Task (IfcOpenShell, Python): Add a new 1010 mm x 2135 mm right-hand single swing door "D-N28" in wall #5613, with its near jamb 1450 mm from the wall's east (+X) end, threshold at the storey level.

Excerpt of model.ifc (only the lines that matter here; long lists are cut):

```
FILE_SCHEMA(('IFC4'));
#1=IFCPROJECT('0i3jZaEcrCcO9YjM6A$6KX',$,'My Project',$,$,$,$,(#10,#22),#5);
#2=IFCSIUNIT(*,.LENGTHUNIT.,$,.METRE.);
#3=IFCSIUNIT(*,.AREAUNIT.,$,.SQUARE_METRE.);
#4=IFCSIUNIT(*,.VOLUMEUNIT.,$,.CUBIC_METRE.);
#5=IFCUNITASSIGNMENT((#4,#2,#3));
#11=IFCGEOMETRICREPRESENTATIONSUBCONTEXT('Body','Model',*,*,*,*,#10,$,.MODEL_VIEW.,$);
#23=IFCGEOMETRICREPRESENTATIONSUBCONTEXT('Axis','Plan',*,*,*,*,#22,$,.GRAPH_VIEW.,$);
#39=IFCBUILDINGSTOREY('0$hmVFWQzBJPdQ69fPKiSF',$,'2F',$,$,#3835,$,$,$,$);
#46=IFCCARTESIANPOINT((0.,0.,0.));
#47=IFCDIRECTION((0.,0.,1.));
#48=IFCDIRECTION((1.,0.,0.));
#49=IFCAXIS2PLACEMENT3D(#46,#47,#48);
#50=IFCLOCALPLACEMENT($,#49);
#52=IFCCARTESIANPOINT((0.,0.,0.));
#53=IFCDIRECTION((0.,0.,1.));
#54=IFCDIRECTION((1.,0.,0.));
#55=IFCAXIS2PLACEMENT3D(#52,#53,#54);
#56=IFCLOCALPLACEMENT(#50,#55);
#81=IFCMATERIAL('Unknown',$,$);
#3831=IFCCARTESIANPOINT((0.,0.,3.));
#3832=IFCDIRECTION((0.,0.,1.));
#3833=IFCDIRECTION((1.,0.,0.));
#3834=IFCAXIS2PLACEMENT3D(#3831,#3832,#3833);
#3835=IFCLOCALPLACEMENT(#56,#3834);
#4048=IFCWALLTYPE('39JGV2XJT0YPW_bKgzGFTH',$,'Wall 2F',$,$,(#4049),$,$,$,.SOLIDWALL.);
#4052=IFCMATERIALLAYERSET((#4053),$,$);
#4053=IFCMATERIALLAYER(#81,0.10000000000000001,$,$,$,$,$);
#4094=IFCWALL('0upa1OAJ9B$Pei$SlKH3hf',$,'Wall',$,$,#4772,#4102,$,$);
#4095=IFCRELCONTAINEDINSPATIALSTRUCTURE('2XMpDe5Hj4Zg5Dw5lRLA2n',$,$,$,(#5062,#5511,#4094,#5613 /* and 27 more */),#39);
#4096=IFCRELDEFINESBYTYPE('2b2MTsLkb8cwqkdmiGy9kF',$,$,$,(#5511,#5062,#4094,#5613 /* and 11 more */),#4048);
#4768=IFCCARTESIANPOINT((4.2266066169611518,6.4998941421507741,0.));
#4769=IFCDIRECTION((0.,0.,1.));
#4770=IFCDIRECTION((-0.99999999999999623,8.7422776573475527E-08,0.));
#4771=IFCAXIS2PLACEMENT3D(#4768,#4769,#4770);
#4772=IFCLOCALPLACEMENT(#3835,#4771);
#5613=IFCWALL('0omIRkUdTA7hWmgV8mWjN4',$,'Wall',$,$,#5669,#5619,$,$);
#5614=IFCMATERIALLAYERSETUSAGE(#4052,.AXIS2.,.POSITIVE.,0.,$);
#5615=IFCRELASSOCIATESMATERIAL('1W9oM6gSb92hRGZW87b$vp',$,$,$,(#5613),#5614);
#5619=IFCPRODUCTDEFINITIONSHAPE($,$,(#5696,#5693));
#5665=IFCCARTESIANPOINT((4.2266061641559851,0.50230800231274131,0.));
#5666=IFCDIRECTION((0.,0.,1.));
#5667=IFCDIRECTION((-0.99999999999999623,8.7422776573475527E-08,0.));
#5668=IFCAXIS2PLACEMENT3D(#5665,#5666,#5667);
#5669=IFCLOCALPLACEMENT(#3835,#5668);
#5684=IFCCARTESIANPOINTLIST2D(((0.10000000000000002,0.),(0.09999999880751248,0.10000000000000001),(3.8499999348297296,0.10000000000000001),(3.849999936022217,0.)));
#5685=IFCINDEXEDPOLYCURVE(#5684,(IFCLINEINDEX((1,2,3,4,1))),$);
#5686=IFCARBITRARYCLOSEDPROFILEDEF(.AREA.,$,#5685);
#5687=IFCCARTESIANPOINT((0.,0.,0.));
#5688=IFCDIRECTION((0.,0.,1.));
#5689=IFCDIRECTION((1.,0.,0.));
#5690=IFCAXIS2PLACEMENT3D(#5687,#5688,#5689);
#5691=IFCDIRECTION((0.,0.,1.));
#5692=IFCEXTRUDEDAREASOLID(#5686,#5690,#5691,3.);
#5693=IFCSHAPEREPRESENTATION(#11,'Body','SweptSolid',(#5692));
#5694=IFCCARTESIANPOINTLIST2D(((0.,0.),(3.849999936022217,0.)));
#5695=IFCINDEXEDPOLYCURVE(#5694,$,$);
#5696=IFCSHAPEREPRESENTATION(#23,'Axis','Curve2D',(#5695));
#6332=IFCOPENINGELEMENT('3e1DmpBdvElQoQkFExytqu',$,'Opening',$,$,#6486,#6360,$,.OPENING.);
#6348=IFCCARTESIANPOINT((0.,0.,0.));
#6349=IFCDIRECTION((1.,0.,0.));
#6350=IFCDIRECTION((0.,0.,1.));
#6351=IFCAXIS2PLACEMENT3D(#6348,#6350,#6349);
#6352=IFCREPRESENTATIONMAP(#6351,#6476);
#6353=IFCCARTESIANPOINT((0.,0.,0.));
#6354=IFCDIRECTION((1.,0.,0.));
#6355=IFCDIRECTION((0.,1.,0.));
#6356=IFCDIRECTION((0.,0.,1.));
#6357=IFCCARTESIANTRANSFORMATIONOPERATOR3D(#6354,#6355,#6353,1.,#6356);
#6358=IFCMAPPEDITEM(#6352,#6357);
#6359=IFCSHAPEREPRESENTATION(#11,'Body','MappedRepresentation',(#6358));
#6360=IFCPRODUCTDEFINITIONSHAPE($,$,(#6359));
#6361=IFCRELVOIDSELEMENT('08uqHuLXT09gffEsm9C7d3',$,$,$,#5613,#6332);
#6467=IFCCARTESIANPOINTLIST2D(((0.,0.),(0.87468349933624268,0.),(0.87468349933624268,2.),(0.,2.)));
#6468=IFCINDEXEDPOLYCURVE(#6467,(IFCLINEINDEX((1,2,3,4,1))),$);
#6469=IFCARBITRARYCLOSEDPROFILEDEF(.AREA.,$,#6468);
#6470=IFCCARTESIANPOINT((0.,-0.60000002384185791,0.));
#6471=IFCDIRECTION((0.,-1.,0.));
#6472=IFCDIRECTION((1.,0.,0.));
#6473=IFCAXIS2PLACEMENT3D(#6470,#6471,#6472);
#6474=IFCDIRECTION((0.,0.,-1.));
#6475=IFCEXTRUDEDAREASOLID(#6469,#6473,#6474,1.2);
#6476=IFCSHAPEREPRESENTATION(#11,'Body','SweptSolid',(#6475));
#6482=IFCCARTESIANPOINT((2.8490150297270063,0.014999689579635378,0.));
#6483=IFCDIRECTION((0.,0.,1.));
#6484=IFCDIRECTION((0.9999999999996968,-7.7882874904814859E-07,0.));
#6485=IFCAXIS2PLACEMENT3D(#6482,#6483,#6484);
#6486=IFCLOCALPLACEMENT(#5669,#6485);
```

```python
import numpy as np
import ifcopenshell
import ifcopenshell.api.feature
import ifcopenshell.api.geometry
import ifcopenshell.api.root
import ifcopenshell.api.spatial
import ifcopenshell.geom
import ifcopenshell.util.element
import ifcopenshell.util.placement
import ifcopenshell.util.representation
import ifcopenshell.util.shape
import ifcopenshell.util.unit

model = ifcopenshell.open("model.ifc")
unit_scale = ifcopenshell.util.unit.calculate_unit_scale(model)
settings = ifcopenshell.geom.settings()


def volume(element):
    """Net volume in cubic metres, openings subtracted."""
    shape = ifcopenshell.geom.create_shape(settings, element)
    return ifcopenshell.util.shape.get_volume(shape.geometry)


wall = model.by_guid("0omIRkUdTA7hWmgV8mWjN4")
storey = ifcopenshell.util.element.get_container(wall, ifc_class="IfcBuildingStorey")
context = ifcopenshell.util.representation.get_context(model, "Model", "Body", "MODEL_VIEW")
before = volume(wall)

width, height, from_end, sill = 1.01, 2.135, 1.45, 0.0  # metres

# The wall runs along its own X axis, and the end named is its -X end.
wall_shape = ifcopenshell.geom.create_shape(settings, wall)
x, y, z = ifcopenshell.util.shape.get_vertices(wall_shape.geometry).T
start = x.min() + from_end
face, thickness = float(y.min()), float(y.max() - y.min())
wall_matrix = ifcopenshell.util.placement.get_local_placement(wall.ObjectPlacement)
level = ifcopenshell.util.placement.get_local_placement(storey.ObjectPlacement)[2, 3]


def in_wall(x, y):
    """Placement at x, y metres in the wall's axes, at sill height."""
    matrix = wall_matrix.copy()
    matrix[:, 3] = wall_matrix @ np.array([x / unit_scale, y / unit_scale, 0.0, 1.0])
    matrix[2, 3] = level + sill / unit_scale
    return matrix


# Opening: a box that overshoots both wall faces by 50 mm.
opening = ifcopenshell.api.root.create_entity(model, ifc_class="IfcOpeningElement", predefined_type="OPENING")
box = ifcopenshell.api.geometry.add_wall_representation(
    model, context=context, length=width, height=height, thickness=thickness + 0.1
)
ifcopenshell.api.geometry.assign_representation(model, product=opening, representation=box)
ifcopenshell.api.geometry.edit_object_placement(model, product=opening, matrix=in_wall(start, face - 0.05), is_si=False)
ifcopenshell.api.feature.add_feature(model, feature=opening, element=wall)

door = ifcopenshell.api.root.create_entity(model, ifc_class="IfcDoor", name="D-N28", predefined_type="DOOR")
door.OverallWidth, door.OverallHeight = width / unit_scale, height / unit_scale
door.OperationType = "SINGLE_SWING_RIGHT"
body = ifcopenshell.api.geometry.add_door_representation(
    model,
    context=context,
    overall_width=door.OverallWidth,
    overall_height=door.OverallHeight,
    operation_type="SINGLE_SWING_RIGHT",
    lining_properties={"LiningDepth": thickness / unit_scale, "ThresholdDepth": thickness / unit_scale},
)
ifcopenshell.api.geometry.assign_representation(model, product=door, representation=body)
ifcopenshell.api.spatial.assign_container(model, products=[door], relating_structure=storey)
ifcopenshell.api.feature.add_filling(model, opening=opening, element=door)

# The lining spans the wall, so the door starts at the wall face.
ifcopenshell.api.geometry.edit_object_placement(model, product=door, matrix=in_wall(start, face), is_si=False)

after = volume(wall)

print(f"wall volume {before:.3f} -> {after:.3f} m3")

model.write("model-out.ifc")
```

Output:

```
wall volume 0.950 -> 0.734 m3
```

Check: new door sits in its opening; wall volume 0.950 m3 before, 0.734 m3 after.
